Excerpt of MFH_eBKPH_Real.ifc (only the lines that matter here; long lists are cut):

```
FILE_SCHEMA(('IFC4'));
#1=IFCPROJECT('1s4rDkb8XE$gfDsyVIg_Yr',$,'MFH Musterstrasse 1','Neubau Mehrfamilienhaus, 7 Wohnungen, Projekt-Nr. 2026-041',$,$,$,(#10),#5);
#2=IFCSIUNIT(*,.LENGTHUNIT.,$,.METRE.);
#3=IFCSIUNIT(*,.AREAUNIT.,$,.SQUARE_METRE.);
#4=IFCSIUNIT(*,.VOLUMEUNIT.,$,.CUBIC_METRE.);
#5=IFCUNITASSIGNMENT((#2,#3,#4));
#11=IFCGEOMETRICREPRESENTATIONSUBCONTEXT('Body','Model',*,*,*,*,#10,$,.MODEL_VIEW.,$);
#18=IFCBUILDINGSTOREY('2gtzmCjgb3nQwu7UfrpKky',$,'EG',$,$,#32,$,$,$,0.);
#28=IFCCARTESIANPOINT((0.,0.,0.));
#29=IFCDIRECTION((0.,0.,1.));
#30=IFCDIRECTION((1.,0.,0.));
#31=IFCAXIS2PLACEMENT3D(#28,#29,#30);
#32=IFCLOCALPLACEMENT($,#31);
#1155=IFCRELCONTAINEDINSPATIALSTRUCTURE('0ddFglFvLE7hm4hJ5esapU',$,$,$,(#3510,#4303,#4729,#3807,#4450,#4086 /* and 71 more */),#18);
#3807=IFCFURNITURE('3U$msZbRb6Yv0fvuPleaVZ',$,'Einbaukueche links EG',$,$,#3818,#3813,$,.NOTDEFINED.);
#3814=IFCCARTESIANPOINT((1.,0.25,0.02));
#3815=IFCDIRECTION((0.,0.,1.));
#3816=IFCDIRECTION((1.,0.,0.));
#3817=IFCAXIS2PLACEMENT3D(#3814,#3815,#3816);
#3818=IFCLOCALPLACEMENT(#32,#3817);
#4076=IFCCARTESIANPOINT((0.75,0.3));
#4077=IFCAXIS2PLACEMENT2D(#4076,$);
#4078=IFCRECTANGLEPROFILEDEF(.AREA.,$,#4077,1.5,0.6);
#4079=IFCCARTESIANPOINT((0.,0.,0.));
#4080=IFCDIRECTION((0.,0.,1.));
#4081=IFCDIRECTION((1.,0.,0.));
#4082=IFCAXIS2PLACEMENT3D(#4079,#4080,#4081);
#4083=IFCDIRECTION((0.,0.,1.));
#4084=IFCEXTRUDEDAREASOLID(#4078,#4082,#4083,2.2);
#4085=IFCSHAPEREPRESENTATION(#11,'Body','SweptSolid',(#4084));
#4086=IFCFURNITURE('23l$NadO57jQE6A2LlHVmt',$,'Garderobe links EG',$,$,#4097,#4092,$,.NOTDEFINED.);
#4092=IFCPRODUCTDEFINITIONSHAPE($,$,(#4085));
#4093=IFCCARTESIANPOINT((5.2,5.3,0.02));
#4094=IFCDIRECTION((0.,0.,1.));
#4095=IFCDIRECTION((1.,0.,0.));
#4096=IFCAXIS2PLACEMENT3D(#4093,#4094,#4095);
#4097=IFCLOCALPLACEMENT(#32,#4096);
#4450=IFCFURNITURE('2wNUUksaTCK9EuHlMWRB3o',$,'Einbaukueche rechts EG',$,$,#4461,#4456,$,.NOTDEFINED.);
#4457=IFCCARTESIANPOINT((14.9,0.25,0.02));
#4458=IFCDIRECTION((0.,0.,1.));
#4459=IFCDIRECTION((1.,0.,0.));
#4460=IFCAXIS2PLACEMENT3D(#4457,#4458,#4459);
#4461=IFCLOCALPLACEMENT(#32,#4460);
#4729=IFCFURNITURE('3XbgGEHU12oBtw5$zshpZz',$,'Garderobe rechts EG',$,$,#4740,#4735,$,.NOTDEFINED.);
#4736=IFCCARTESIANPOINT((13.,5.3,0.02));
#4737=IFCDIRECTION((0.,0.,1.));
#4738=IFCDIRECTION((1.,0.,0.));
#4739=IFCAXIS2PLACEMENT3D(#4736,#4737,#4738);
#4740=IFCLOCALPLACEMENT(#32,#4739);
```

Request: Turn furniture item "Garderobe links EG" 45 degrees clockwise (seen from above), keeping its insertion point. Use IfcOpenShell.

```python
import ifcopenshell
import ifcopenshell.api.geometry
import ifcopenshell.util.placement

model = ifcopenshell.open("MFH_eBKPH_Real.ifc")

item = model.by_id(4086)
matrix = ifcopenshell.util.placement.get_local_placement(item.ObjectPlacement)
matrix = matrix @ ifcopenshell.util.placement.rotation(-45, "Z")
ifcopenshell.api.geometry.edit_object_placement(model, product=item, matrix=matrix, is_si=False)

print(ifcopenshell.util.placement.get_local_placement(item.ObjectPlacement).round(3) + 0.0)

model.write("MFH_eBKPH_Real-out.ifc")
```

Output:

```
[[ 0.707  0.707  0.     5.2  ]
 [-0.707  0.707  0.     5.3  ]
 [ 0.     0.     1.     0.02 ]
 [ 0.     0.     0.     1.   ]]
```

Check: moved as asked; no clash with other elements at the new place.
